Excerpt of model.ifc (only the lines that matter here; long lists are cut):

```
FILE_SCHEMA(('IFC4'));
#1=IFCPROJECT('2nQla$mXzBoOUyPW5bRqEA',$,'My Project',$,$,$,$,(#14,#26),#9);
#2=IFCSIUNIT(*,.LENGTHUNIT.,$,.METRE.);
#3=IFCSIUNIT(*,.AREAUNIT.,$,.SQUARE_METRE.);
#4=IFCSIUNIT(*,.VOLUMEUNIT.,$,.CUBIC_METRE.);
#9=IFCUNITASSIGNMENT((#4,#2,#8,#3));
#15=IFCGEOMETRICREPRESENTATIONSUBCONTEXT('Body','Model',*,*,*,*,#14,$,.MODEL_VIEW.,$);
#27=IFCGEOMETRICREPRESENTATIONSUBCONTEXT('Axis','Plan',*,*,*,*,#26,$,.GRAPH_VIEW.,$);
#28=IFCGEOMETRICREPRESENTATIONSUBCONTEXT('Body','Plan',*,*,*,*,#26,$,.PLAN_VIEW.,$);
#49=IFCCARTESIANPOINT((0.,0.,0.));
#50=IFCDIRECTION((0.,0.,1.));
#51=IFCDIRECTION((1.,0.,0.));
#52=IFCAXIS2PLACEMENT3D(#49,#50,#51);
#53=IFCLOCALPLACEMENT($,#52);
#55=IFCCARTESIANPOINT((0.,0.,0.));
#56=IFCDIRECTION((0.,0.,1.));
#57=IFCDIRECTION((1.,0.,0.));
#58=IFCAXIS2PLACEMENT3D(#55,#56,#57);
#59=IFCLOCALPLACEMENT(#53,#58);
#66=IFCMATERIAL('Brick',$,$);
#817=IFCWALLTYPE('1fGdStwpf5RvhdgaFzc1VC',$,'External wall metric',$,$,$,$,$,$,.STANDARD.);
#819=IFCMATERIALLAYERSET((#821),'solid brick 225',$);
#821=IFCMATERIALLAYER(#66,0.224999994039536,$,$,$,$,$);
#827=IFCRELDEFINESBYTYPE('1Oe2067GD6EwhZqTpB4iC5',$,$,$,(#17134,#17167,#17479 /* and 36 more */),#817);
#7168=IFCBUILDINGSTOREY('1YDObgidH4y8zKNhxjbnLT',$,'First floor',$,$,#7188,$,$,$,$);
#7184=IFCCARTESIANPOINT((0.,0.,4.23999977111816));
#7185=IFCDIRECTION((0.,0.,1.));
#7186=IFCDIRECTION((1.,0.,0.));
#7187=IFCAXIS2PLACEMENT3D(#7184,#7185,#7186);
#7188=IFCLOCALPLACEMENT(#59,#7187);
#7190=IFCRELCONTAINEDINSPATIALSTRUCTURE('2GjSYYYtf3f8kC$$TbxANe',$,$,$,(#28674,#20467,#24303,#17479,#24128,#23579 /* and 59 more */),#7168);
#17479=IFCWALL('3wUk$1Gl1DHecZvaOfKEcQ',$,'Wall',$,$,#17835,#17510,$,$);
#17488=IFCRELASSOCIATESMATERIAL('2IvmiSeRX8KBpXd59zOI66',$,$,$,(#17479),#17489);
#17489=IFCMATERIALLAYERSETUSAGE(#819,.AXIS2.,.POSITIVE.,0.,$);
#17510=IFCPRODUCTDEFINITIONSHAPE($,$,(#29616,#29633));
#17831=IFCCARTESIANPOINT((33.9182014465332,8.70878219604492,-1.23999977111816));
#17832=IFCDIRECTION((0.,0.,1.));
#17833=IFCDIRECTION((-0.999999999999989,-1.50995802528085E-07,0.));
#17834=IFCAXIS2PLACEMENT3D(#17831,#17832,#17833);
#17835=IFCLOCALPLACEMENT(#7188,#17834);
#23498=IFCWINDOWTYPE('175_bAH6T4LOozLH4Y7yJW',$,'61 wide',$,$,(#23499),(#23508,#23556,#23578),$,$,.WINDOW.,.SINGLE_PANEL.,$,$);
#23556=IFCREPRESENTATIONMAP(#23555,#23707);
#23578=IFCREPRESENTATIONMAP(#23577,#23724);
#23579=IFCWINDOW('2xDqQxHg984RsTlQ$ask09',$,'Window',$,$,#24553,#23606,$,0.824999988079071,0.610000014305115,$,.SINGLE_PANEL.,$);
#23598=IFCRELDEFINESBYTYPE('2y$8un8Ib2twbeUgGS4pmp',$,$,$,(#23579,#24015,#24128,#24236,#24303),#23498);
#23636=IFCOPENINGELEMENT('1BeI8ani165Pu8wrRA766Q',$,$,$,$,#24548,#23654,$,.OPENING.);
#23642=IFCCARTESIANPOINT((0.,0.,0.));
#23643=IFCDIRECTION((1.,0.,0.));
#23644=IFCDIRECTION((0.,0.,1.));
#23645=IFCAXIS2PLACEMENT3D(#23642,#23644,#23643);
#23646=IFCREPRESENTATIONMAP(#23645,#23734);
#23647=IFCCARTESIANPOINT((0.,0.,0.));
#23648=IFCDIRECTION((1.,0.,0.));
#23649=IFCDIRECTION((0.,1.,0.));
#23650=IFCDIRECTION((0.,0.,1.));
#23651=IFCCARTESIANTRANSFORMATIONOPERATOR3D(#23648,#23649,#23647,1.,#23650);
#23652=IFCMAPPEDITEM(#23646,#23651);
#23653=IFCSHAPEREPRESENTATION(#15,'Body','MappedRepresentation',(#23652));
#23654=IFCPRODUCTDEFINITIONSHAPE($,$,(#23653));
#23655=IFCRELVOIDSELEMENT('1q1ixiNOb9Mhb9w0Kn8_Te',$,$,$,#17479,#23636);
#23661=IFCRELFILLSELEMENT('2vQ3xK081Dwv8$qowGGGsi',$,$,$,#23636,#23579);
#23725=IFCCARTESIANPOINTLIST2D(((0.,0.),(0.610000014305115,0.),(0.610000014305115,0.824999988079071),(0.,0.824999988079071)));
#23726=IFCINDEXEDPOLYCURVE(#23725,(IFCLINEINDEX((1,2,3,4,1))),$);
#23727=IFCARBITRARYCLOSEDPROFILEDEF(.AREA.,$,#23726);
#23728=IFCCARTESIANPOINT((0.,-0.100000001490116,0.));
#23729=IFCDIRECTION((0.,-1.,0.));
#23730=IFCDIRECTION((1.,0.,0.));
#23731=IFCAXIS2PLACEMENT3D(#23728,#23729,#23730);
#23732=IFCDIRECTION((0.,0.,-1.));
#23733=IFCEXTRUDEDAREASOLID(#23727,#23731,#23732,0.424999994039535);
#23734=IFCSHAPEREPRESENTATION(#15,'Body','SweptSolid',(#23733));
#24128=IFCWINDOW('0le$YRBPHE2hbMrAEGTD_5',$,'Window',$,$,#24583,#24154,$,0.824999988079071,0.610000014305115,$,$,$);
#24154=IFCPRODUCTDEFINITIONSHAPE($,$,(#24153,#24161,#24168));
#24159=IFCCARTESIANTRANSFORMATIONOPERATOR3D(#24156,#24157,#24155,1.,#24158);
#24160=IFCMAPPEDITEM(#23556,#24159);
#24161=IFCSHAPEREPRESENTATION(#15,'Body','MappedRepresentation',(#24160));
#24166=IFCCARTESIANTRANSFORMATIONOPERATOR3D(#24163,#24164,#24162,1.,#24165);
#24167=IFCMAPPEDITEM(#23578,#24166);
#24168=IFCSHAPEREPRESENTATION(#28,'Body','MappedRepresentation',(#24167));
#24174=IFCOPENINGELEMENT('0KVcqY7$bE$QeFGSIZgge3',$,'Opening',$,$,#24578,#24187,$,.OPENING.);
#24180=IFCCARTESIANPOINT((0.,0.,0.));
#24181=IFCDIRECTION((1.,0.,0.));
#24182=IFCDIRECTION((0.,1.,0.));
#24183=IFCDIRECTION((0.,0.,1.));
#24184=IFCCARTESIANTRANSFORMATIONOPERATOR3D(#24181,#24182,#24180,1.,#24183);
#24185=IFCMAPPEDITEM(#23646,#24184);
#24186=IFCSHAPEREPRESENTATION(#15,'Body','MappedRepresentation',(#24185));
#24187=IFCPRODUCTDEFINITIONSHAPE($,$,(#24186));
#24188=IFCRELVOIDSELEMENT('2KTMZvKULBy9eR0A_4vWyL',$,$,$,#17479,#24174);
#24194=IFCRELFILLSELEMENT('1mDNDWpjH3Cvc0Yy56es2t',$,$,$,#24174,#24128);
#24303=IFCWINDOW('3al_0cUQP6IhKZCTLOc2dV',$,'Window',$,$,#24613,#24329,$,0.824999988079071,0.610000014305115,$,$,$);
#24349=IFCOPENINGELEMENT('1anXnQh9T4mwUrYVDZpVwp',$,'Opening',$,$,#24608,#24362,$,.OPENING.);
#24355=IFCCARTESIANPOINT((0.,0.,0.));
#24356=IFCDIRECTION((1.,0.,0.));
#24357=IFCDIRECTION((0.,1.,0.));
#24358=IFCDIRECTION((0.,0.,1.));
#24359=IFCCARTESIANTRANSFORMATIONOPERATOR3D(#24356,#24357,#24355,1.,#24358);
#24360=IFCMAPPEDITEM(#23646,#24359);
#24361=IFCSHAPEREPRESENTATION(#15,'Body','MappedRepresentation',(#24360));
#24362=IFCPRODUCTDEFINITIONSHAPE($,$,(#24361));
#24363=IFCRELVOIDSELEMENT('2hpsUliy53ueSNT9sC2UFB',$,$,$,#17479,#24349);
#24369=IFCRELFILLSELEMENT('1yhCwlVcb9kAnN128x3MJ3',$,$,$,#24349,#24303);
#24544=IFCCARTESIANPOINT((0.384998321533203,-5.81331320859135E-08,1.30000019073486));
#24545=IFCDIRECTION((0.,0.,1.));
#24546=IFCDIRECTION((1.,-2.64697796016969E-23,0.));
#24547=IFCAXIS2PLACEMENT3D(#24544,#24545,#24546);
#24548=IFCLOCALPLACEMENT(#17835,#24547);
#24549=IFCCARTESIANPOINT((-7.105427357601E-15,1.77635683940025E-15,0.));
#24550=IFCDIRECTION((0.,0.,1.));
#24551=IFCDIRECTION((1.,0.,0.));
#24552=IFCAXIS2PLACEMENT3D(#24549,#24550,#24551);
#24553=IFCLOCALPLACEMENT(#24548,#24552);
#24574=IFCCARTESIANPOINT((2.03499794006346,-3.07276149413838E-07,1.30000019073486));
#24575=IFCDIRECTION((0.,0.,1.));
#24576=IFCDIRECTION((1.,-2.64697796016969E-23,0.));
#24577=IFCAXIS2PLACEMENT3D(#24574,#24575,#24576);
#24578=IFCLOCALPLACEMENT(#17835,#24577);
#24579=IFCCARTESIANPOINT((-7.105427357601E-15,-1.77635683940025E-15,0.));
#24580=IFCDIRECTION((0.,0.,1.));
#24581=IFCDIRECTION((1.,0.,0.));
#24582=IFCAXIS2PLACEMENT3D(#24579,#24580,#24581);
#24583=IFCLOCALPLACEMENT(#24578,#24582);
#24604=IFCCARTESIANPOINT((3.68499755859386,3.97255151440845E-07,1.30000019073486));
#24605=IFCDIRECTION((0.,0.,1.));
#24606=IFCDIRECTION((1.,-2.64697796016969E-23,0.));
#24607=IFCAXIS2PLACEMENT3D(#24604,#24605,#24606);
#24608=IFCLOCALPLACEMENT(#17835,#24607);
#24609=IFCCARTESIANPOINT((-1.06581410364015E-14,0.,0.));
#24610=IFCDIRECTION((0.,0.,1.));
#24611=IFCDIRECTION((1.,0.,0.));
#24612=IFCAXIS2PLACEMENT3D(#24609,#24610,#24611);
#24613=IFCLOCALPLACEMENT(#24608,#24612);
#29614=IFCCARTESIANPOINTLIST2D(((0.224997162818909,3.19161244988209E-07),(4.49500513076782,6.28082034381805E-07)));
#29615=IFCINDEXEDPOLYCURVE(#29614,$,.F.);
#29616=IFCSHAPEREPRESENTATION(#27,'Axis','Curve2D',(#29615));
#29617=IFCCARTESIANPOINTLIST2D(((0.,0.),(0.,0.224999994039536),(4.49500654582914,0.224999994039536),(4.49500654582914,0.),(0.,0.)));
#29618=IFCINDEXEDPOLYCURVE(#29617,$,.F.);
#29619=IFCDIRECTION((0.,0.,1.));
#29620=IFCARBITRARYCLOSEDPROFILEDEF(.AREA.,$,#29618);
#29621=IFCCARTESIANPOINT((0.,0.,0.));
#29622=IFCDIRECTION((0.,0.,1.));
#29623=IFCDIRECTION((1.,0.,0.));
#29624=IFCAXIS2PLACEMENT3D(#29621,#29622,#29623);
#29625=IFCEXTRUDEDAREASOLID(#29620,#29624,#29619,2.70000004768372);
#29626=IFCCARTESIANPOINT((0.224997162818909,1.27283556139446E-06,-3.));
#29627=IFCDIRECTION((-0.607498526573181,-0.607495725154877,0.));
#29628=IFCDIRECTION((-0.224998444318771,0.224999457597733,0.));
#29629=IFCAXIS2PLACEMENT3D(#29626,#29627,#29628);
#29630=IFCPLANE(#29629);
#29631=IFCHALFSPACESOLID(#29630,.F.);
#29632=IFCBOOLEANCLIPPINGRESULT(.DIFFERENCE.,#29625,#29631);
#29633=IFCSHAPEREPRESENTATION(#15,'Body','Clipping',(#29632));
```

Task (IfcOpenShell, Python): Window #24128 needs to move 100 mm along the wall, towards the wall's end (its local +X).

```python
import ifcopenshell
import ifcopenshell.api.geometry
import ifcopenshell.util.placement
import ifcopenshell.util.unit

model = ifcopenshell.open("model.ifc")
unit_scale = ifcopenshell.util.unit.calculate_unit_scale(model)

window = model.by_guid("0le$YRBPHE2hbMrAEGTD_5")
opening = window.FillsVoids[0].RelatingOpeningElement
wall = opening.VoidsElements[0].RelatingBuildingElement

wall_matrix = ifcopenshell.util.placement.get_local_placement(wall.ObjectPlacement)
shift = wall_matrix[:3, 0] * 0.1 / unit_scale
before = ifcopenshell.util.placement.get_local_placement(window.ObjectPlacement)[:3, 3].copy()

# The window is placed relative to its opening, so it follows when the opening moves.
matrix = ifcopenshell.util.placement.get_local_placement(opening.ObjectPlacement)
matrix[:3, 3] += shift
ifcopenshell.api.geometry.edit_object_placement(
    model, product=opening, matrix=matrix, is_si=False, should_transform_children=True
)

after = ifcopenshell.util.placement.get_local_placement(window.ObjectPlacement)[:3, 3]
print("window moved by", (after - before).round(3) + 0.0)

model.write("model_edited.ifc")
```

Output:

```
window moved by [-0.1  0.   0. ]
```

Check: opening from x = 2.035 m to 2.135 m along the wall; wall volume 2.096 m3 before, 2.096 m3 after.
